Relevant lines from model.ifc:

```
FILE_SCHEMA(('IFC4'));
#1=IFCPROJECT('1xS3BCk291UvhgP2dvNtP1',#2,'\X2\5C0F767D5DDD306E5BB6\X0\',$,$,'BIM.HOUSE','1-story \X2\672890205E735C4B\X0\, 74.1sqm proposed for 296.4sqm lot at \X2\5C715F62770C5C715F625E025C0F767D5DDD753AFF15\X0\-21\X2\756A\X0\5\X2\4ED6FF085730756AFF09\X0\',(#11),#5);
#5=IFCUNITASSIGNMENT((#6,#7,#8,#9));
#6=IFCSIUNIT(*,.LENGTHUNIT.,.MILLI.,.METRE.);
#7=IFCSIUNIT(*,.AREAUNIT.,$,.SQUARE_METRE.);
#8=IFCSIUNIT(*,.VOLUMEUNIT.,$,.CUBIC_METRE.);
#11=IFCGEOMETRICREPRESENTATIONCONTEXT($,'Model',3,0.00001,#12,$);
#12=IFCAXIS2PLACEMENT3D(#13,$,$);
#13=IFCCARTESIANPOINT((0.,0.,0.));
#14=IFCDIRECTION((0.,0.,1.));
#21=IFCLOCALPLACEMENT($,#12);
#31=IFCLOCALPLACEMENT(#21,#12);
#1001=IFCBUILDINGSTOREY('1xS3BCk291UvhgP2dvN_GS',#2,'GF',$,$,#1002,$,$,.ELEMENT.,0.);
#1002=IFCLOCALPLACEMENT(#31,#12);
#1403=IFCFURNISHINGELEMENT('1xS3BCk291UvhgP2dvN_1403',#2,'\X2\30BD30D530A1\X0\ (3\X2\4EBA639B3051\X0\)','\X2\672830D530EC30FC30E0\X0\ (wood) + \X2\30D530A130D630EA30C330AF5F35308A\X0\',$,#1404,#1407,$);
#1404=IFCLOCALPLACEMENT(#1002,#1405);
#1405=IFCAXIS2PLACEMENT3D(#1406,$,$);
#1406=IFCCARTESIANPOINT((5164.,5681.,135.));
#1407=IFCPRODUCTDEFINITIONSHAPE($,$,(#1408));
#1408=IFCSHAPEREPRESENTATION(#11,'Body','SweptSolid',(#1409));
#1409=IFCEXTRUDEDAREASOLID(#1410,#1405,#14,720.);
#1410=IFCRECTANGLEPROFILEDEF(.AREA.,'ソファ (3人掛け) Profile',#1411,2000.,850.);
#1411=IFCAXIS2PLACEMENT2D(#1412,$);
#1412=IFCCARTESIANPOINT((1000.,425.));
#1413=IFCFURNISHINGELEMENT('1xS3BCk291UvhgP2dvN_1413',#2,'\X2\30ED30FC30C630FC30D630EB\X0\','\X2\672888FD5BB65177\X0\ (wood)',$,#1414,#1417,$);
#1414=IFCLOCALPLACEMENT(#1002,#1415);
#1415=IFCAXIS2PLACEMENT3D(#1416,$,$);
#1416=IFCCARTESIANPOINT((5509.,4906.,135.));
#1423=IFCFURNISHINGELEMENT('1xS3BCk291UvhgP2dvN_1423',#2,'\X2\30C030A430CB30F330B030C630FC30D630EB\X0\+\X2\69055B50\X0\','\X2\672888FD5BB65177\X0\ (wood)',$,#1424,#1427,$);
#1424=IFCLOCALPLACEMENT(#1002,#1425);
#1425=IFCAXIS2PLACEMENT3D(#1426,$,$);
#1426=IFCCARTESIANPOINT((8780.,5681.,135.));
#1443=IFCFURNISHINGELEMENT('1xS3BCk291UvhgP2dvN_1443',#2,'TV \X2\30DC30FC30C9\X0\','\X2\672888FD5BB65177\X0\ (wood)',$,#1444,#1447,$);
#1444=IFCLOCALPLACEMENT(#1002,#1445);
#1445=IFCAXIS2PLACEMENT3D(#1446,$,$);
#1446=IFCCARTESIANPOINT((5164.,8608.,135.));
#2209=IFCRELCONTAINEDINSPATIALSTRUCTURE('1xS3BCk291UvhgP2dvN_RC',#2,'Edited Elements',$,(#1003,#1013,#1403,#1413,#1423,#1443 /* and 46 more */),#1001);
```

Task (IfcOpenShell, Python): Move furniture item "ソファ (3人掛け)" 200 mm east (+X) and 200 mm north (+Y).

```python
import ifcopenshell
import ifcopenshell.api.geometry
import ifcopenshell.util.placement

model = ifcopenshell.open("model.ifc")

item = model.by_guid("1xS3BCk291UvhgP2dvN_1403")
matrix = ifcopenshell.util.placement.get_local_placement(item.ObjectPlacement)
matrix[0, 3] += 200.0
matrix[1, 3] += 200.0
ifcopenshell.api.geometry.edit_object_placement(model, product=item, matrix=matrix, is_si=False)

print(ifcopenshell.util.placement.get_local_placement(item.ObjectPlacement).round(3) + 0.0)

model.write("model_rev.ifc")
```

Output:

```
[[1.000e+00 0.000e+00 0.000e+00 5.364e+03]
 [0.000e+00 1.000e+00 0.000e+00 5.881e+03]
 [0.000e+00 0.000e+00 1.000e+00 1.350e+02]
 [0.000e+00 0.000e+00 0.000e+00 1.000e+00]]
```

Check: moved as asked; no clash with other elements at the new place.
